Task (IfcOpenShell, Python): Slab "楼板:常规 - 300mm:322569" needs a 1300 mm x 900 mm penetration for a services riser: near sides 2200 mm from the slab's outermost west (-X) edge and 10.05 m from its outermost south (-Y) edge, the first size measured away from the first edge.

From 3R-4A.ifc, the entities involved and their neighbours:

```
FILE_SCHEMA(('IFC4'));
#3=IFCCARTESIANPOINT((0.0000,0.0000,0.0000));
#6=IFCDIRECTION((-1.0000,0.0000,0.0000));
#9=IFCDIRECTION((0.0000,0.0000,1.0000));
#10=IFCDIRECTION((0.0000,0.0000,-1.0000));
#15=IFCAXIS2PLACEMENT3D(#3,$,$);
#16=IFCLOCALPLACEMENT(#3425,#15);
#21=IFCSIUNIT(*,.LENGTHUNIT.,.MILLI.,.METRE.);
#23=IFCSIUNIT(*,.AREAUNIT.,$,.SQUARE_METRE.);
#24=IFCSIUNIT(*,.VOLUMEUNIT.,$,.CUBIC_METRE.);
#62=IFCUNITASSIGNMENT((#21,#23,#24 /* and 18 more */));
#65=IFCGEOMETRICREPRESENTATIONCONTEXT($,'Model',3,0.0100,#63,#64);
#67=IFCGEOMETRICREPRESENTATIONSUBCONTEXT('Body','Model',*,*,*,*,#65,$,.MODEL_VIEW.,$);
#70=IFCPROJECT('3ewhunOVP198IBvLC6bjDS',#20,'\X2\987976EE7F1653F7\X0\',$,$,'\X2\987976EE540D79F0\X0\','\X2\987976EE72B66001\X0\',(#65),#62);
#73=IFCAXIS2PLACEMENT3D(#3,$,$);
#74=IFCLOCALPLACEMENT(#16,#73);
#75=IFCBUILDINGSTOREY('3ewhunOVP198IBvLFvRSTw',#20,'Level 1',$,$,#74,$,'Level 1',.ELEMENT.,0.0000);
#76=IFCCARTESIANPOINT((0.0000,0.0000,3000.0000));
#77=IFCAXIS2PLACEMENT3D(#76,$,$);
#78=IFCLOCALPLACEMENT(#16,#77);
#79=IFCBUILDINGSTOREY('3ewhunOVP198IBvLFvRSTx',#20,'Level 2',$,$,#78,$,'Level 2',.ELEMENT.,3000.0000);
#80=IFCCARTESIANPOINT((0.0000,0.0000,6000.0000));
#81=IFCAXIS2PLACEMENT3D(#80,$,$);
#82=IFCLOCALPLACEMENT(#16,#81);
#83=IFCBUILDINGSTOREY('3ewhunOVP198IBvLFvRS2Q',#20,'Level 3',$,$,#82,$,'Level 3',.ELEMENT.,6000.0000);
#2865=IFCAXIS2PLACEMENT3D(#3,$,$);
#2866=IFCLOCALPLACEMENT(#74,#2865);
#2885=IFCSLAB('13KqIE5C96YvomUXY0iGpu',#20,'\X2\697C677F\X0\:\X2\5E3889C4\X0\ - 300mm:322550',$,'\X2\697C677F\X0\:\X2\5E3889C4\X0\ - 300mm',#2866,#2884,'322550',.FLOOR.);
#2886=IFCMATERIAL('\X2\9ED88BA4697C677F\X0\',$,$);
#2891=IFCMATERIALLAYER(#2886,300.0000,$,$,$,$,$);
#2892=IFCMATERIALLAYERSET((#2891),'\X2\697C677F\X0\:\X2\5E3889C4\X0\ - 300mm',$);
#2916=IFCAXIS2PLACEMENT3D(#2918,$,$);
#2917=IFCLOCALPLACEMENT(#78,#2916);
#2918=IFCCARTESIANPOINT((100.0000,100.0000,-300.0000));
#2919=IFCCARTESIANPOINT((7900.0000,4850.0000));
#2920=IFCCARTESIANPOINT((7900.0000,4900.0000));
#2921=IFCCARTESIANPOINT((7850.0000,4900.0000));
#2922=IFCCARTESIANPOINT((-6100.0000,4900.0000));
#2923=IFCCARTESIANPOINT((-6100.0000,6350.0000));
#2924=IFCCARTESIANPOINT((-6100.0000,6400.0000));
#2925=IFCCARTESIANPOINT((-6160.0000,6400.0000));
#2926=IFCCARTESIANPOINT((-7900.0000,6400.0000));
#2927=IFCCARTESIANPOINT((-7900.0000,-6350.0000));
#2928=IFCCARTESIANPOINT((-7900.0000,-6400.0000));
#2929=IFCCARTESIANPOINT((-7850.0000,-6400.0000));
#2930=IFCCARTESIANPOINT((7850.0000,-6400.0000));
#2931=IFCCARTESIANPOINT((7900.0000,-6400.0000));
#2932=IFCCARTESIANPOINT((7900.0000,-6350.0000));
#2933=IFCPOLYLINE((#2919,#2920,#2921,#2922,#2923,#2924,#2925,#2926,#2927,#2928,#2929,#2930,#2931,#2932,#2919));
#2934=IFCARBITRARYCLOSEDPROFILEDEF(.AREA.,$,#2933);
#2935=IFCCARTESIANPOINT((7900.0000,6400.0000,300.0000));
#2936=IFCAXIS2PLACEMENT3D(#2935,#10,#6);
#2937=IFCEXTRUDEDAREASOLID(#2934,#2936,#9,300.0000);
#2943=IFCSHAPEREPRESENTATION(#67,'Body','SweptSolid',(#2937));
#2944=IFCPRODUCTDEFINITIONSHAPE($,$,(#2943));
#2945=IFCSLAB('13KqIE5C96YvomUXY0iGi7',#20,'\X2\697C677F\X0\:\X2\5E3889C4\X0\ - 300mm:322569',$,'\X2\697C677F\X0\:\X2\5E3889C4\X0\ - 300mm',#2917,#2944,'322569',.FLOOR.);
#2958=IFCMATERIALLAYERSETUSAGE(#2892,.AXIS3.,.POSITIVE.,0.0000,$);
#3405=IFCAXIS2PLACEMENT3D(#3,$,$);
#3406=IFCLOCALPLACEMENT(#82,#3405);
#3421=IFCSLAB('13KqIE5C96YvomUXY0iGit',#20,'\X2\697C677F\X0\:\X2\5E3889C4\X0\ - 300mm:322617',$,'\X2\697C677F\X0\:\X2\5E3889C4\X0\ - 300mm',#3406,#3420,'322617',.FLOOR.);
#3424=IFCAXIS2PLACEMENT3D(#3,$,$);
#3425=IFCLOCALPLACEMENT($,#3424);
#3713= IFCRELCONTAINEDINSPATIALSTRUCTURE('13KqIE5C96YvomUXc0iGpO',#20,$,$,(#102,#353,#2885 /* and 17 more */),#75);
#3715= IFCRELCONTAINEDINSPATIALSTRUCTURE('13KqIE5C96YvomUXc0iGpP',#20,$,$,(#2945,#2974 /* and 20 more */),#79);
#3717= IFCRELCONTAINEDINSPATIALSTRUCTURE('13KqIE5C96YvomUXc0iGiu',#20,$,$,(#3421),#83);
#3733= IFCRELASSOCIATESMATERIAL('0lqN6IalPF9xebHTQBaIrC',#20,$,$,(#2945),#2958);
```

```python
import numpy as np
import ifcopenshell
import ifcopenshell.api.feature
import ifcopenshell.api.geometry
import ifcopenshell.api.root
import ifcopenshell.geom
import ifcopenshell.util.placement
import ifcopenshell.util.representation
import ifcopenshell.util.shape
import ifcopenshell.util.unit

model = ifcopenshell.open("3R-4A.ifc")
unit_scale = ifcopenshell.util.unit.calculate_unit_scale(model)
settings = ifcopenshell.geom.settings()


def volume(element):
    """Net volume in cubic metres, openings subtracted."""
    shape = ifcopenshell.geom.create_shape(settings, element)
    return ifcopenshell.util.shape.get_volume(shape.geometry)


slab = model.by_guid("13KqIE5C96YvomUXY0iGi7")
before = volume(slab)

# Extent in the slab's own axes, in metres. The edges named are its -X and -Y sides.
slab_shape = ifcopenshell.geom.create_shape(settings, slab)
vertices = ifcopenshell.util.shape.get_vertices(slab_shape.geometry)
x_min, y_min, bottom = vertices.min(axis=0)
top = vertices[:, 2].max()

opening = ifcopenshell.api.root.create_entity(model, ifc_class="IfcOpeningElement", name="Services riser opening", predefined_type="OPENING")
context = ifcopenshell.util.representation.get_context(model, "Model", "Body", "MODEL_VIEW")
width, depth = 1.3, 0.9
outline = [(0.0, 0.0), (width, 0.0), (width, depth), (0.0, depth), (0.0, 0.0)]
# Overshoot both faces by 50 mm so the cut is clean.
shape = ifcopenshell.api.geometry.add_slab_representation(
    model, context=context, depth=top - bottom + 0.1, polyline=outline
)
ifcopenshell.api.geometry.assign_representation(model, product=opening, representation=shape)

matrix = ifcopenshell.util.placement.get_local_placement(slab.ObjectPlacement)
matrix[:, 3] = matrix @ np.append(np.array([x_min + 2.2, y_min + 10.05, bottom - 0.05]) / unit_scale, 1.0)
ifcopenshell.api.geometry.edit_object_placement(model, product=opening, matrix=matrix, is_si=False)
ifcopenshell.api.feature.add_feature(model, feature=opening, element=slab)

after = volume(slab)

print(f"slab volume {before:.3f} -> {after:.3f} m3")

model.write("3R-4A_v2.ifc")
```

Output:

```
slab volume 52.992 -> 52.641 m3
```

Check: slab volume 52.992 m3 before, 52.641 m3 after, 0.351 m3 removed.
